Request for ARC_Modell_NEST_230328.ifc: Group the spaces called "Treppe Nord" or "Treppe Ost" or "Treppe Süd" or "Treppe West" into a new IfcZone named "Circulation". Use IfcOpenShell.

First a look at what the model holds.

```python
import ifcopenshell

model = ifcopenshell.open("ARC_Modell_NEST_230328.ifc")
print(model.schema)
seen = {}
for space in model.by_type("IfcSpace"):
    seen[space.LongName] = seen.get(space.LongName, 0) + 1
for name, count in sorted(seen.items(), key=str):
    print(count, "x", name)
print("zones:", [z.Name for z in model.by_type("IfcZone")][:20])
```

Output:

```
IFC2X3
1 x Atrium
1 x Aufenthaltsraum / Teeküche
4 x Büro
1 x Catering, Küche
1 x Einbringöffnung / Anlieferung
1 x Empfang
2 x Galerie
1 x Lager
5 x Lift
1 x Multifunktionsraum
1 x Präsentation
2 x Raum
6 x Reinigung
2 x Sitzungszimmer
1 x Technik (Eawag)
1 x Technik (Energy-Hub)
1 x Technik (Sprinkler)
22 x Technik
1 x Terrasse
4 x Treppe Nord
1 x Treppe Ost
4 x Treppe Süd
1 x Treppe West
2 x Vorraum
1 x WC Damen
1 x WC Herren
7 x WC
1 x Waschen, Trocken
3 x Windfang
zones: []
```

```python
import ifcopenshell
import ifcopenshell.api.group
import ifcopenshell.api.root

model = ifcopenshell.open("ARC_Modell_NEST_230328.ifc")

names = {"Treppe Nord", "Treppe Ost", "Treppe Süd", "Treppe West"}
spaces = [s for s in model.by_type("IfcSpace") if s.LongName in names]

zone = ifcopenshell.api.root.create_entity(model, ifc_class="IfcZone", name="Circulation")
ifcopenshell.api.group.assign_group(model, products=spaces, group=zone)
print(len(spaces), "spaces in", zone.Name)

model.write("ARC_Modell_NEST_230328_updated.ifc")
```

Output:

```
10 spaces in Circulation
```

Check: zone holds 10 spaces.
